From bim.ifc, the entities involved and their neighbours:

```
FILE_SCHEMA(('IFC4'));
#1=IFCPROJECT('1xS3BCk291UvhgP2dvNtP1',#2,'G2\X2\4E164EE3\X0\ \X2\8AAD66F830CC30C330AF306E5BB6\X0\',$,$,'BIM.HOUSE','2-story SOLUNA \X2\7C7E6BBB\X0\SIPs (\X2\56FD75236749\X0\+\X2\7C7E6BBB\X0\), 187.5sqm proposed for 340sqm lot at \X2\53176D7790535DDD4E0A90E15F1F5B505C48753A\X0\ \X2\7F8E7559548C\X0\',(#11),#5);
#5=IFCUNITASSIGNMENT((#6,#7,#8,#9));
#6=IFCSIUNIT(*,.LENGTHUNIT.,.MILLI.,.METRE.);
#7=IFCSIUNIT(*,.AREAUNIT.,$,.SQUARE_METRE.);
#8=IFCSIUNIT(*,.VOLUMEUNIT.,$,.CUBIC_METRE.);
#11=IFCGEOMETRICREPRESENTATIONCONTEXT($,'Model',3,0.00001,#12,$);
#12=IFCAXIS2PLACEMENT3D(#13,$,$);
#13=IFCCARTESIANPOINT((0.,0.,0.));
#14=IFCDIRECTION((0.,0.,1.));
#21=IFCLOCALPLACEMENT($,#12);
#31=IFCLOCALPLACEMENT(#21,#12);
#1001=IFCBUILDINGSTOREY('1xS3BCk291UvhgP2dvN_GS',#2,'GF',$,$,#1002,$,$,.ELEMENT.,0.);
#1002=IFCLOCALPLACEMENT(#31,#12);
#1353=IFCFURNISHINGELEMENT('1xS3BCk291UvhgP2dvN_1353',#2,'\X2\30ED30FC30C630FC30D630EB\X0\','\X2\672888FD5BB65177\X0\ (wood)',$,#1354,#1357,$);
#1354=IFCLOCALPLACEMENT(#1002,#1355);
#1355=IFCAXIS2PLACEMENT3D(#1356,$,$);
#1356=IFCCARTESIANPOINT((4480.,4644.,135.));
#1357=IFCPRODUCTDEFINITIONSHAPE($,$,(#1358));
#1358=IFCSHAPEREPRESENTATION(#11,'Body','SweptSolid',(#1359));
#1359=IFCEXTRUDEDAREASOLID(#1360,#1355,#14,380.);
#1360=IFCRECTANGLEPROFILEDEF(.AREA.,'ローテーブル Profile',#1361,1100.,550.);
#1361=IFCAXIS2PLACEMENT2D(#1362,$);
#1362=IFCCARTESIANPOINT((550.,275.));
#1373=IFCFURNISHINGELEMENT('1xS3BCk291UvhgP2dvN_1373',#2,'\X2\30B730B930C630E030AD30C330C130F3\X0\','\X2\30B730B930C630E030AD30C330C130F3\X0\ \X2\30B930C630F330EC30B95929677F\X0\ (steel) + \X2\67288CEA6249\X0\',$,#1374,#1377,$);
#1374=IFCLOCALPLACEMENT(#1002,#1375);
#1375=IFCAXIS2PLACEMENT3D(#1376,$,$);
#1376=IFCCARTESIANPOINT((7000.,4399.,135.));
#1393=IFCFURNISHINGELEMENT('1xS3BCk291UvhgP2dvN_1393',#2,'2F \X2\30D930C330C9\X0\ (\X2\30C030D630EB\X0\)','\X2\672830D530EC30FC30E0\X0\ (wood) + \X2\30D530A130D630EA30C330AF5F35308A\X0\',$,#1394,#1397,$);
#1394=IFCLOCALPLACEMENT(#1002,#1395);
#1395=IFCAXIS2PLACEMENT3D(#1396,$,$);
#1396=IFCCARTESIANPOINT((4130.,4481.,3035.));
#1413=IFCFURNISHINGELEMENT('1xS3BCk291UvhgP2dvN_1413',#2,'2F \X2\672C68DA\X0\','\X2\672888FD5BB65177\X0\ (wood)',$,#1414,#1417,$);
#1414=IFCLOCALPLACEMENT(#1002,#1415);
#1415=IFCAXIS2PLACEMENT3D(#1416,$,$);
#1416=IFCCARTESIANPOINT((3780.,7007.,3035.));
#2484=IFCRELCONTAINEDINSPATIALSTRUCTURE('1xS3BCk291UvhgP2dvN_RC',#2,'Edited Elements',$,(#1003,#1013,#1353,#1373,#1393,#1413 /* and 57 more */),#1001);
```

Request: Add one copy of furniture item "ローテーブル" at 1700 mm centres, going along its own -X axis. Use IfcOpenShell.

```python
import ifcopenshell
import ifcopenshell.api.geometry
import ifcopenshell.api.root
import ifcopenshell.util.element
import ifcopenshell.util.placement

model = ifcopenshell.open("bim.ifc")


def reuse_history(source, copy):
    """copy_class also copies each property set's owner history, people and application; keep the originals."""
    for rel in copy.IsDefinedBy:
        if rel.is_a("IfcRelDefinesByProperties") and (history := rel.RelatingPropertyDefinition.OwnerHistory):
            rel.RelatingPropertyDefinition.OwnerHistory = source.OwnerHistory
            ifcopenshell.util.element.remove_deep2(model, history)


source = model.by_guid("1xS3BCk291UvhgP2dvN_1353")
base = ifcopenshell.util.placement.get_local_placement(source.ObjectPlacement)
step = -base[:3, 0] * 1700.0

for i in range(1, 2):
    copy = ifcopenshell.api.root.copy_class(model, product=source)
    copy.Representation = ifcopenshell.util.element.copy_deep(
        model, source.Representation, exclude=["IfcGeometricRepresentationContext", "IfcRepresentationMap"]
    )
    reuse_history(source, copy)
    matrix = base.copy()
    matrix[:3, 3] += i * step
    print("added at", matrix[:3, 3].round(3) + 0.0)
    ifcopenshell.api.geometry.edit_object_placement(model, product=copy, matrix=matrix, is_si=False)

model.write("bim_updated.ifc")
```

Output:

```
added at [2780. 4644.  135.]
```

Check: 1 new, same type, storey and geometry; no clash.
